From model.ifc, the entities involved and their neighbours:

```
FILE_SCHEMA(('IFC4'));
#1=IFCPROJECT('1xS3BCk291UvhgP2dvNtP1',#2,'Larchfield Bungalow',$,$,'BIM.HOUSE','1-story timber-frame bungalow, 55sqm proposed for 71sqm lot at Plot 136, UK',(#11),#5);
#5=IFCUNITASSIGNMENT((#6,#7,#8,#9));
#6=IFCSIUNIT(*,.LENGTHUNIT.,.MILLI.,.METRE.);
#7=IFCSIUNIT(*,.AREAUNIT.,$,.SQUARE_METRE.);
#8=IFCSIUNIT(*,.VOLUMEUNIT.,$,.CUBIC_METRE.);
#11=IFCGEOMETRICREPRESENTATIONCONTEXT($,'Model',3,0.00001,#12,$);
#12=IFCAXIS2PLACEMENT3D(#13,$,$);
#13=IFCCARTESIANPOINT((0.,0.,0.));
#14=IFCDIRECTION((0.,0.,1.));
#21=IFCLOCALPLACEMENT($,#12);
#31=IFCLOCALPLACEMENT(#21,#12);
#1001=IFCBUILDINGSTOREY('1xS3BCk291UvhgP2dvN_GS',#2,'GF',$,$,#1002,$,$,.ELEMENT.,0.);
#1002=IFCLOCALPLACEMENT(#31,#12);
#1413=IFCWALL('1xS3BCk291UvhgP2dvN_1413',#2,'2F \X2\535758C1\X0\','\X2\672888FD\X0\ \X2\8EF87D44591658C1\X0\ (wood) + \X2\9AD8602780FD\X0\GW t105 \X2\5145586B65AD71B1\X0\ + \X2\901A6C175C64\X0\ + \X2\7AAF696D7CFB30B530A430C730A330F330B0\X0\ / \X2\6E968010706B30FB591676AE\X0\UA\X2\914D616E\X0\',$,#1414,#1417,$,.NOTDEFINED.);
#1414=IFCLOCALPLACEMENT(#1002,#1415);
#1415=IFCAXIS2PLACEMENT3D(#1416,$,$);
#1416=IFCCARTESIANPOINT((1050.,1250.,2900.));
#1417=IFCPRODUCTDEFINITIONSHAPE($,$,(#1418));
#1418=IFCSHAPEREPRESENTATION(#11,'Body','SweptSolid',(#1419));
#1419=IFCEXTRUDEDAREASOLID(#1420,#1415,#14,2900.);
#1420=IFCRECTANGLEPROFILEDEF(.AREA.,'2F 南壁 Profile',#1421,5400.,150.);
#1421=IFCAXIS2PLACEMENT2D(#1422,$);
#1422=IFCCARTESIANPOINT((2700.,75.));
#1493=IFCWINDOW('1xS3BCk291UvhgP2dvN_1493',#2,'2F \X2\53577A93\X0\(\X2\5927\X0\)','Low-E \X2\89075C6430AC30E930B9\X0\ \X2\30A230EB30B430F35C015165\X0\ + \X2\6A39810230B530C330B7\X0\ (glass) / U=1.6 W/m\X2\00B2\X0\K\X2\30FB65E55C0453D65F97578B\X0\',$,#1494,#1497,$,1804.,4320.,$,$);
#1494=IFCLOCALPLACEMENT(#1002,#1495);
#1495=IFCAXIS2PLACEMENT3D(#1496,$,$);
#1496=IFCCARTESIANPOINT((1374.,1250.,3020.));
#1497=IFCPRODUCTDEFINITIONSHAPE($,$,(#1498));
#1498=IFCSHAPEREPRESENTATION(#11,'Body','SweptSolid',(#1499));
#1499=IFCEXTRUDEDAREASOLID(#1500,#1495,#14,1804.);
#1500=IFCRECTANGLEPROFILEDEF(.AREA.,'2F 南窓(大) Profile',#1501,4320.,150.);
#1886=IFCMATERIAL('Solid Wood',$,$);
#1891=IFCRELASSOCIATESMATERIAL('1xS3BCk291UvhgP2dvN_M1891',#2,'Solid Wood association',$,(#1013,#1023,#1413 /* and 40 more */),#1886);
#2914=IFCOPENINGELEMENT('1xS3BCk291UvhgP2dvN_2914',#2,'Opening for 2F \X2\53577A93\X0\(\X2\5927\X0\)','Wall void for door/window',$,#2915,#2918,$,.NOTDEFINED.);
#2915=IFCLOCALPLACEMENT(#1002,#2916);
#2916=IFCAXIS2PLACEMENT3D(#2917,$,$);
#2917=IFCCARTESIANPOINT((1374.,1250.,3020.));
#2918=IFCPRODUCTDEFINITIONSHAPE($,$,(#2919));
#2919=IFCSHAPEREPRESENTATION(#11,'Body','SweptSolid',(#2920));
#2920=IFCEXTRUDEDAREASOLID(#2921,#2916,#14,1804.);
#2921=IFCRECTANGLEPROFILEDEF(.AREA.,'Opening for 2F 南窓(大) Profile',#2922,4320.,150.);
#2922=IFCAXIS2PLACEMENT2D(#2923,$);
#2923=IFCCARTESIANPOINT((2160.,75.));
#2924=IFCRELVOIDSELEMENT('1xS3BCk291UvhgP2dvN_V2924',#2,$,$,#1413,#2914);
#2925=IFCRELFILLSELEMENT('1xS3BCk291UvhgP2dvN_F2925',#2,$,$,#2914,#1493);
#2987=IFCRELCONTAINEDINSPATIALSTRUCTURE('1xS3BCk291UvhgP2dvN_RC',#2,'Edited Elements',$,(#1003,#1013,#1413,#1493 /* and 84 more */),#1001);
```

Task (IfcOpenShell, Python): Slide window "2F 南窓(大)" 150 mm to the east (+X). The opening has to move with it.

```python
import ifcopenshell
import ifcopenshell.api.geometry
import ifcopenshell.util.placement

model = ifcopenshell.open("model.ifc")

window = model.by_id(1493)
opening = window.FillsVoids[0].RelatingOpeningElement
wall = opening.VoidsElements[0].RelatingBuildingElement

wall_matrix = ifcopenshell.util.placement.get_local_placement(wall.ObjectPlacement)
shift = wall_matrix[:3, 0] * 150.0
before = ifcopenshell.util.placement.get_local_placement(window.ObjectPlacement)[:3, 3].copy()

# The window is not placed relative to its opening, so move both.
for product in (opening, window):
    matrix = ifcopenshell.util.placement.get_local_placement(product.ObjectPlacement)
    matrix[:3, 3] += shift
    ifcopenshell.api.geometry.edit_object_placement(model, product=product, matrix=matrix, is_si=False)

after = ifcopenshell.util.placement.get_local_placement(window.ObjectPlacement)[:3, 3]
print("window moved by", (after - before).round(3) + 0.0)

model.write("model_edited.ifc")
```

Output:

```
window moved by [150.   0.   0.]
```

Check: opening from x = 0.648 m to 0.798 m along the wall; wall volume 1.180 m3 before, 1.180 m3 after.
